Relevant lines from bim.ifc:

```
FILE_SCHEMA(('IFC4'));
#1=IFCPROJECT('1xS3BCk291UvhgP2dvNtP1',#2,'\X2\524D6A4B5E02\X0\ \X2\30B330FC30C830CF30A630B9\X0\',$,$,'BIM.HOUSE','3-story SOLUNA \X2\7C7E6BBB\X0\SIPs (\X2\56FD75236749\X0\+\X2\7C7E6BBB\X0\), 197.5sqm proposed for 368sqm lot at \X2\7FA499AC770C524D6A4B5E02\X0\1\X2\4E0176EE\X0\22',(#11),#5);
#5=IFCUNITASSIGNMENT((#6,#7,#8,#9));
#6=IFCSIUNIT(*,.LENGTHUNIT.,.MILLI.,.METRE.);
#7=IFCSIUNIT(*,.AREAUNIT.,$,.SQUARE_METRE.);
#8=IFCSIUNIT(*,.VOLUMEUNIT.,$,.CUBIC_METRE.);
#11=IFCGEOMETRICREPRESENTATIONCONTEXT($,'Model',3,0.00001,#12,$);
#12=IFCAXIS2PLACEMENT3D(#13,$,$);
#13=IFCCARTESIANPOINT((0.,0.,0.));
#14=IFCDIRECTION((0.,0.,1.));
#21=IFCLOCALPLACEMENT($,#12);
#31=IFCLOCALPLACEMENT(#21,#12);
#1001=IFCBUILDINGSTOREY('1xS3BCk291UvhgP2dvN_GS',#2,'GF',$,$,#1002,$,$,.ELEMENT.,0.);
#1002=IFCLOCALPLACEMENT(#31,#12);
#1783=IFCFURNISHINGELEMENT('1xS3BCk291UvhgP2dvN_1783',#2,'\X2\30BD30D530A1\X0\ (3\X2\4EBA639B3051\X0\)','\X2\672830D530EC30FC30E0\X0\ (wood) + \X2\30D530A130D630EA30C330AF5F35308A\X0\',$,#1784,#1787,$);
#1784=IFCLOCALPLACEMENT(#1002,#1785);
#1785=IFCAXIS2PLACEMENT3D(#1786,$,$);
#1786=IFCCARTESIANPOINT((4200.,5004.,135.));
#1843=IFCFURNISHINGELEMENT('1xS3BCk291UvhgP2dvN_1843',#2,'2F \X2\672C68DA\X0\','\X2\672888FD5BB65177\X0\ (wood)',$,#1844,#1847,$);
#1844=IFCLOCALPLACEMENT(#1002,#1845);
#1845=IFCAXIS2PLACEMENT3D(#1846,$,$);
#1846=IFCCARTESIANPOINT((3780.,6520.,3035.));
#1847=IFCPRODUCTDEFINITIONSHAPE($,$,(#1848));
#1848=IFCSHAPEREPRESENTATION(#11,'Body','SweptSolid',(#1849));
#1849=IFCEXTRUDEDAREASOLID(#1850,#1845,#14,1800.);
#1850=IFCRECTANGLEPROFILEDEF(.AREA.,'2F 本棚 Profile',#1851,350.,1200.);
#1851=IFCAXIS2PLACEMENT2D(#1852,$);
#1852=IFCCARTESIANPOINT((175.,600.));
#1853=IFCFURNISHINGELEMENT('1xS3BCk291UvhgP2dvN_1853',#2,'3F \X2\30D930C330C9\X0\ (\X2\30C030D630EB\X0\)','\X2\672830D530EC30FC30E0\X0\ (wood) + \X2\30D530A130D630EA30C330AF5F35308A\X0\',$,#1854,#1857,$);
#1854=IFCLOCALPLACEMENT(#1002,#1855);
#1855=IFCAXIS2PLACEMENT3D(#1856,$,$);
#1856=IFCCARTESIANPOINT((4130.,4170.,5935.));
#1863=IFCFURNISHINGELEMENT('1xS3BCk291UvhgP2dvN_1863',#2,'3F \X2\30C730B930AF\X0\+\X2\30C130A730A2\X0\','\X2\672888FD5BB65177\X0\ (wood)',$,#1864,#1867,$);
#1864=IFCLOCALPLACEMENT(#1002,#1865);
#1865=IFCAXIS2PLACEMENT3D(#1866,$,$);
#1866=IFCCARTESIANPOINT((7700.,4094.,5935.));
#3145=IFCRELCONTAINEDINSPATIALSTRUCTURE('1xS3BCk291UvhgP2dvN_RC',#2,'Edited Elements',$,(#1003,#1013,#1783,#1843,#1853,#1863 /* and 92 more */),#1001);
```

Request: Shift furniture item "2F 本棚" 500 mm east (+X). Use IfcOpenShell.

```python
import ifcopenshell
import ifcopenshell.api.geometry
import ifcopenshell.util.placement

model = ifcopenshell.open("bim.ifc")

item = model.by_id(1843)
matrix = ifcopenshell.util.placement.get_local_placement(item.ObjectPlacement)
matrix[0, 3] += 500.0
ifcopenshell.api.geometry.edit_object_placement(model, product=item, matrix=matrix, is_si=False)

print(ifcopenshell.util.placement.get_local_placement(item.ObjectPlacement).round(3) + 0.0)

model.write("bim-out.ifc")
```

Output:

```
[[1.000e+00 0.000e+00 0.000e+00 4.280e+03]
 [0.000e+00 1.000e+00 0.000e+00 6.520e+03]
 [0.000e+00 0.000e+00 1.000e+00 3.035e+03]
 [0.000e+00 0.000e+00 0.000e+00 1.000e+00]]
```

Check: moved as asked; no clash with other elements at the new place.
